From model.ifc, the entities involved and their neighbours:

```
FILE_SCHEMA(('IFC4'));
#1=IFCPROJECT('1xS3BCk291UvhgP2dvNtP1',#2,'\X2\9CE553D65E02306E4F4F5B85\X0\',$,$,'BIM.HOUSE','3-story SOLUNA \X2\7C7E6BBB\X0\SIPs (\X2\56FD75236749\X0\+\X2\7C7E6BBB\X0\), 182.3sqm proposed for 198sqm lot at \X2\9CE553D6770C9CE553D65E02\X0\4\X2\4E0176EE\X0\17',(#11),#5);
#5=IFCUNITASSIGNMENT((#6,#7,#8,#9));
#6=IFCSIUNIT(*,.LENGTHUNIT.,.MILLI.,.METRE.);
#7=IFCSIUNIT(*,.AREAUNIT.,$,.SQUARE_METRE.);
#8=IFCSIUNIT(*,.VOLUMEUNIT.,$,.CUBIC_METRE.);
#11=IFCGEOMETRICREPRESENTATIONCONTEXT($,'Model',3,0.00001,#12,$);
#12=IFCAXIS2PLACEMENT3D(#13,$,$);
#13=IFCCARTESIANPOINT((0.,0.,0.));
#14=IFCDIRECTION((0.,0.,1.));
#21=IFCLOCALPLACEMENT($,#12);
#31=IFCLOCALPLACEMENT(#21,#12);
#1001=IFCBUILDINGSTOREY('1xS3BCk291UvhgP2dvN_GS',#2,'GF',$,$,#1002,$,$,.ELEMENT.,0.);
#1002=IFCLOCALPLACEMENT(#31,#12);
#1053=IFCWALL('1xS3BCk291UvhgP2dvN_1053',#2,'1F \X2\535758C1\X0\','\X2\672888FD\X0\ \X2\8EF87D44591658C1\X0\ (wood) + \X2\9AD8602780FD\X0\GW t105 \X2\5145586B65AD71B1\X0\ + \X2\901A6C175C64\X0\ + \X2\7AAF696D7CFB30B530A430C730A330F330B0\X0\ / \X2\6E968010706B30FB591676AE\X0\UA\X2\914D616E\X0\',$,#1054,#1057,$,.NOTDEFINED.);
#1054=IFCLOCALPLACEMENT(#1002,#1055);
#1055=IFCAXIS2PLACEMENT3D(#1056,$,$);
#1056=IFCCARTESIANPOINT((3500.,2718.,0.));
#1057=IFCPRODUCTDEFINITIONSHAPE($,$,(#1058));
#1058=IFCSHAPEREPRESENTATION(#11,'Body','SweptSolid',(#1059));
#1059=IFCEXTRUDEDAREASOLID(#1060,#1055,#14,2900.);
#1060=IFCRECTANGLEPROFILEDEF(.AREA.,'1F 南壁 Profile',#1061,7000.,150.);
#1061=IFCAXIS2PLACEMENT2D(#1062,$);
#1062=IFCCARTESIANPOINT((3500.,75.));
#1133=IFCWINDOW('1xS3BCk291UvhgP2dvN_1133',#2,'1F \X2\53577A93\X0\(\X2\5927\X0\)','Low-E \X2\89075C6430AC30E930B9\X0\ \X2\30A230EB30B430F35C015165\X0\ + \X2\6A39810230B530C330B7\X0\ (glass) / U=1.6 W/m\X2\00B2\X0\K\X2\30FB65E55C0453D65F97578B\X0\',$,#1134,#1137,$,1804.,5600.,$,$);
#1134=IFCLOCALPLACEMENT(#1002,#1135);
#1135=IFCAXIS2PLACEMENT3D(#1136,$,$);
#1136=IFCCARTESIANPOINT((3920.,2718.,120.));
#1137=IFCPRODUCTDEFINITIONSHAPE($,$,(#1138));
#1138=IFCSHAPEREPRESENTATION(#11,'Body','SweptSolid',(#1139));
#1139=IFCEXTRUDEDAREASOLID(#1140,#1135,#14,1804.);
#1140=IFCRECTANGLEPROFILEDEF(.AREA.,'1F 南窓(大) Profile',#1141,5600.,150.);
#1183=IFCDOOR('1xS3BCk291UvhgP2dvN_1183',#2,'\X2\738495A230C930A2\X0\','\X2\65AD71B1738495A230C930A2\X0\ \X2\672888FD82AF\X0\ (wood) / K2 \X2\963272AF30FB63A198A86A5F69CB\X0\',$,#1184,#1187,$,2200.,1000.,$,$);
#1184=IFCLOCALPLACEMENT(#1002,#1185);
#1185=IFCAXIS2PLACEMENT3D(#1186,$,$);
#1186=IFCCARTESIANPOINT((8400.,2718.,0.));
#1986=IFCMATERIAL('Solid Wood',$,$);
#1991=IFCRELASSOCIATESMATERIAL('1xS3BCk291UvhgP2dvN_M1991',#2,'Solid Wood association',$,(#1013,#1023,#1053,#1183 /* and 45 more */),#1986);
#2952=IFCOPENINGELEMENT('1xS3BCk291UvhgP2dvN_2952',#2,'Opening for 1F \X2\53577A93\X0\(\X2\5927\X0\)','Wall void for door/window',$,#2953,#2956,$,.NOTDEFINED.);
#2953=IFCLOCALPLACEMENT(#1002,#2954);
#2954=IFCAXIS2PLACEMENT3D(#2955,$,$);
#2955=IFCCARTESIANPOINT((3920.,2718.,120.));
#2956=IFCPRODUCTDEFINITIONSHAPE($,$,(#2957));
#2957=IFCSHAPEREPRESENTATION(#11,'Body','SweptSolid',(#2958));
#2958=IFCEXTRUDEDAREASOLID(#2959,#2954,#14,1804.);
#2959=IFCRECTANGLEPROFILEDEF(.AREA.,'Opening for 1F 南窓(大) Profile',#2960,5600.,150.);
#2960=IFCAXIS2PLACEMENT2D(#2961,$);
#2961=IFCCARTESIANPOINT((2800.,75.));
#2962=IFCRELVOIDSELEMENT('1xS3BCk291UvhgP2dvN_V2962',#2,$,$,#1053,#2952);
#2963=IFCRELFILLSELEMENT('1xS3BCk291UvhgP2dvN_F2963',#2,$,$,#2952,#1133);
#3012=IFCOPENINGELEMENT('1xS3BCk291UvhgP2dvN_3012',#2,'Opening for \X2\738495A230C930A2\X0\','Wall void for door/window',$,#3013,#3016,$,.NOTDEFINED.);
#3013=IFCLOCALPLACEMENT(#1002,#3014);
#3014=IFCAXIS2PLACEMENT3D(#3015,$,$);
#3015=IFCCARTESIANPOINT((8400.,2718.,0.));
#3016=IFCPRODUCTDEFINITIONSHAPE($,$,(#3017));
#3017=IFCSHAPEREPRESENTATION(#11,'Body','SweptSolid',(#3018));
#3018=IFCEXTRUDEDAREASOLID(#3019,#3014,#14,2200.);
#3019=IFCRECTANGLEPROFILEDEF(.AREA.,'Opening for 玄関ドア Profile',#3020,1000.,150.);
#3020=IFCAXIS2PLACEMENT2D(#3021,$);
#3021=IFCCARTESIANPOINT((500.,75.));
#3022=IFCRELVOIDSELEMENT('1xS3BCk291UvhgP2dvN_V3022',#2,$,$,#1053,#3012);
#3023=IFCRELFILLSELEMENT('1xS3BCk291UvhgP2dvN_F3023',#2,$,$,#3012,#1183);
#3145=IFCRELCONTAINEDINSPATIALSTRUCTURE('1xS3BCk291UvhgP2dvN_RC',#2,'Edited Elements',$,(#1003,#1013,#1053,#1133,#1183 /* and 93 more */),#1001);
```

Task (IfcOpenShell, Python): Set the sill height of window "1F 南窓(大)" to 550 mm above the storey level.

```python
import numpy as np
import ifcopenshell
import ifcopenshell.api.geometry
import ifcopenshell.geom
import ifcopenshell.util.element
import ifcopenshell.util.placement
import ifcopenshell.util.shape
import ifcopenshell.util.unit

model = ifcopenshell.open("model.ifc")
unit_scale = ifcopenshell.util.unit.calculate_unit_scale(model)

window = model.by_guid("1xS3BCk291UvhgP2dvN_1133")
opening = window.FillsVoids[0].RelatingOpeningElement
storey = ifcopenshell.util.element.get_container(window, ifc_class="IfcBuildingStorey")
level = ifcopenshell.util.placement.get_local_placement(storey.ObjectPlacement)[2, 3]

# The opening's origin need not be at the sill, so measure its lowest point.
shape = ifcopenshell.geom.create_shape(ifcopenshell.geom.settings(), opening)
bottom = ifcopenshell.util.shape.get_shape_bottom_elevation(shape, shape.geometry) / unit_scale
dz = level + 0.55 / unit_scale - bottom

shift = np.array([0.0, 0.0, dz])
# The window is not placed relative to its opening, so move both.
for product in (opening, window):
    matrix = ifcopenshell.util.placement.get_local_placement(product.ObjectPlacement)
    matrix[:3, 3] += shift
    ifcopenshell.api.geometry.edit_object_placement(model, product=product, matrix=matrix, is_si=False)

print(f"moved by {dz * unit_scale:+.3f} m")

model.write("model_edited.ifc")
```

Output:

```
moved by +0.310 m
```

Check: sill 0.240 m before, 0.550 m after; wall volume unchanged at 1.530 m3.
